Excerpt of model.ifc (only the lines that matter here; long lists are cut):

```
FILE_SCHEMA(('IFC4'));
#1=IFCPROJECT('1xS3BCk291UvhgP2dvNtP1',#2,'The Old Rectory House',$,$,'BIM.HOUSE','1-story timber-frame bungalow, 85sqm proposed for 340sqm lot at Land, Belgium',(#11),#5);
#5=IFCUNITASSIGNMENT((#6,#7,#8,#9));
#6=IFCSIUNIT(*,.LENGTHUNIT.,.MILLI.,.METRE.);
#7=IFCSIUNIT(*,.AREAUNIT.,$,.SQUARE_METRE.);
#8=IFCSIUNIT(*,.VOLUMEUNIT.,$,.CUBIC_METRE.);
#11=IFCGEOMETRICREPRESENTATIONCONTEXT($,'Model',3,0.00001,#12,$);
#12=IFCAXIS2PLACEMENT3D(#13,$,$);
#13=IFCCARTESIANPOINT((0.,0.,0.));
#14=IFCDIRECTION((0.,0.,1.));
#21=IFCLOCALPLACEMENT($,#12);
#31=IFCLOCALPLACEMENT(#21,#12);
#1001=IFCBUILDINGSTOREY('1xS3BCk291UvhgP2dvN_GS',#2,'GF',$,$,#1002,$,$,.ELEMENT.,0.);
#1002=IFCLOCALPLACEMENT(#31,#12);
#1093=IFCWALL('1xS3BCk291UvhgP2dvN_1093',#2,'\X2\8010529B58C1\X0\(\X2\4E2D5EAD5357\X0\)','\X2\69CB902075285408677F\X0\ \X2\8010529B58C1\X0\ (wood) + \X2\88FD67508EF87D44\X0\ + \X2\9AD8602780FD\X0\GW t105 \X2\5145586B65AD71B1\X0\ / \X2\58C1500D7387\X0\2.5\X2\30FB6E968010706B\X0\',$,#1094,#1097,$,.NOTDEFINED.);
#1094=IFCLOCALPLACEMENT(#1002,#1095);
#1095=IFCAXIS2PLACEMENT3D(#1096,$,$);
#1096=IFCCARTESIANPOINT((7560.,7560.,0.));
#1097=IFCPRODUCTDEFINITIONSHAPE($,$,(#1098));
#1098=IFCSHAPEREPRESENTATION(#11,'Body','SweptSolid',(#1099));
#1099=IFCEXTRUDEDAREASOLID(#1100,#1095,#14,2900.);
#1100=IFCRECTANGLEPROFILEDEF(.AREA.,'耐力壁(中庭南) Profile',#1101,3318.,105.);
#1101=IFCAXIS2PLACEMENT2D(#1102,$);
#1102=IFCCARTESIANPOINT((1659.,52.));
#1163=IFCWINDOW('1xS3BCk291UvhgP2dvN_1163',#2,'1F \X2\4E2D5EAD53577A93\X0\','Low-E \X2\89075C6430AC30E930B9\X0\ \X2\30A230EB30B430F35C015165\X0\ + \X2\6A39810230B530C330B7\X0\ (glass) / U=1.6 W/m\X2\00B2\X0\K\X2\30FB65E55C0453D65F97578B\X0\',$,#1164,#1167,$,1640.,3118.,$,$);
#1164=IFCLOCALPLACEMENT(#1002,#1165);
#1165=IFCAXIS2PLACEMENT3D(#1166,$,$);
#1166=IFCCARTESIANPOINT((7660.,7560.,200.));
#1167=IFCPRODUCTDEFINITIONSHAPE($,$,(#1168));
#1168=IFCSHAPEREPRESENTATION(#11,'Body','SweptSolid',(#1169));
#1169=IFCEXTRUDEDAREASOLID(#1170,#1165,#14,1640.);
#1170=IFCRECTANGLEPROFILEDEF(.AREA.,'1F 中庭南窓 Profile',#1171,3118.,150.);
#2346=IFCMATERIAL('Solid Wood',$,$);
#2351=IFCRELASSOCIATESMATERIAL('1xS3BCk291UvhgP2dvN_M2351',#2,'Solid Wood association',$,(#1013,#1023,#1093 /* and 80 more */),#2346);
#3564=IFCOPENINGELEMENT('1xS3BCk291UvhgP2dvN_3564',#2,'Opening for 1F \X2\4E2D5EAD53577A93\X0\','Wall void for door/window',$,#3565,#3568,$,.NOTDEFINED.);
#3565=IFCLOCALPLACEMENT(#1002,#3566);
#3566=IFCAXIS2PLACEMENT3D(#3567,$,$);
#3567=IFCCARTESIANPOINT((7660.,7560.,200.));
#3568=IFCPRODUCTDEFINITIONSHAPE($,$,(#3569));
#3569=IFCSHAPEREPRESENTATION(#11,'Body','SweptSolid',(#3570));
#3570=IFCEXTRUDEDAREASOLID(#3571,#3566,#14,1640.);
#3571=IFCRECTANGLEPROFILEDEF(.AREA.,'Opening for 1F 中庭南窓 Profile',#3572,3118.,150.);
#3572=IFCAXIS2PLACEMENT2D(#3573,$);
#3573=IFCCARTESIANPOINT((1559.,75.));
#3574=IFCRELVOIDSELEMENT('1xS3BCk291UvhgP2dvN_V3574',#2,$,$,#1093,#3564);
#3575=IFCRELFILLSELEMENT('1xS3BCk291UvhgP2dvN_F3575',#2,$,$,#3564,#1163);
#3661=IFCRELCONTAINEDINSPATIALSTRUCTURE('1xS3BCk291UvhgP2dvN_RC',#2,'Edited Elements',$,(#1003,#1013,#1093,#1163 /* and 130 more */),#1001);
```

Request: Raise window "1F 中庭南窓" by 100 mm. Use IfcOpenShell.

```python
import numpy as np
import ifcopenshell
import ifcopenshell.api.geometry
import ifcopenshell.util.placement
import ifcopenshell.util.unit

model = ifcopenshell.open("model.ifc")
unit_scale = ifcopenshell.util.unit.calculate_unit_scale(model)

window = model.by_guid("1xS3BCk291UvhgP2dvN_1163")
opening = window.FillsVoids[0].RelatingOpeningElement
dz = 100.0

shift = np.array([0.0, 0.0, dz])
# The window is not placed relative to its opening, so move both.
for product in (opening, window):
    matrix = ifcopenshell.util.placement.get_local_placement(product.ObjectPlacement)
    matrix[:3, 3] += shift
    ifcopenshell.api.geometry.edit_object_placement(model, product=product, matrix=matrix, is_si=False)

print(f"moved by {dz * unit_scale:+.3f} m")

model.write("model_edited.ifc")
```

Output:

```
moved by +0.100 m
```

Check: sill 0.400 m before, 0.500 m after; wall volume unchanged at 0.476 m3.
